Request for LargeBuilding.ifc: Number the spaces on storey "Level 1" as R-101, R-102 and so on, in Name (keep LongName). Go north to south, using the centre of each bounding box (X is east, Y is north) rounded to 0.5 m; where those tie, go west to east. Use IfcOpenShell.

First a look at what the model holds.

```python
import ifcopenshell
import ifcopenshell.util.element
import ifcopenshell.util.placement

model = ifcopenshell.open("LargeBuilding.ifc")
print(model.schema)
storey = next(s for s in model.by_type("IfcBuildingStorey") if s.Name == "Level 1")
spaces = [e for e in ifcopenshell.util.element.get_decomposition(storey) if e.is_a("IfcSpace")]
for e in sorted(spaces, key=lambda e: e.id()):
    origin = ifcopenshell.util.placement.get_local_placement(e.ObjectPlacement)[:3, 3]
    print(e.id(), e.Name, e.LongName, origin.round(2) + 0.0, sep=" | ")
```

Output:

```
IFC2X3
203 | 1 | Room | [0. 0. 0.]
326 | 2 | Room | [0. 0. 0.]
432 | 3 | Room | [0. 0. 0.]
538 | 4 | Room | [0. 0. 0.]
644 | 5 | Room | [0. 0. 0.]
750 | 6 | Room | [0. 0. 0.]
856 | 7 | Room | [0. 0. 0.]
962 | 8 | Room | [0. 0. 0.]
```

```python
import ifcopenshell
import ifcopenshell.geom
import ifcopenshell.util.element
import ifcopenshell.util.shape

model = ifcopenshell.open("LargeBuilding.ifc")
settings = ifcopenshell.geom.settings()
settings.set("use-world-coords", True)


def centre(element):
    shape = ifcopenshell.geom.create_shape(settings, element)
    return ifcopenshell.util.shape.get_bbox_centroid(shape.geometry)


storey = next(s for s in model.by_type("IfcBuildingStorey") if s.Name == "Level 1")
spaces = [e for e in ifcopenshell.util.element.get_decomposition(storey) if e.is_a("IfcSpace")]

# Insertion points can sit at a corner or the storey origin, so sort by the geometry (in metres).
centres = {e: centre(e) for e in spaces}
spaces.sort(key=lambda e: (-round(centres[e][1] / 0.5), centres[e][0]))

for i, e in enumerate(spaces, start=1):
    number = f"R-1{i:02d}"
    e.Name = number
    print(e.id(), number)

model.write("LargeBuilding_rev.ifc")
```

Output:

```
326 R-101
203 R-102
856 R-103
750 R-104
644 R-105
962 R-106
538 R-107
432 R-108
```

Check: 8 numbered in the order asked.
